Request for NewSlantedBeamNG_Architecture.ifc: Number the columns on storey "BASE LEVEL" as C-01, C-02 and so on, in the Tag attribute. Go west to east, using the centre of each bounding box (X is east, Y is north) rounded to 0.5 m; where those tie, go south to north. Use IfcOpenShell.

First a look at what the model holds.

```python
import ifcopenshell
import ifcopenshell.util.element
import ifcopenshell.util.placement

model = ifcopenshell.open("NewSlantedBeamNG_Architecture.ifc")
print(model.schema)
storey = next(s for s in model.by_type("IfcBuildingStorey") if s.Name == "BASE LEVEL")
columns = [e for e in ifcopenshell.util.element.get_decomposition(storey) if e.is_a("IfcColumn")]
for e in sorted(columns, key=lambda e: e.id()):
    origin = ifcopenshell.util.placement.get_local_placement(e.ObjectPlacement)[:3, 3]
    print(e.id(), e.Tag, e.Name, origin.round(2) + 0.0, sep=" | ")
```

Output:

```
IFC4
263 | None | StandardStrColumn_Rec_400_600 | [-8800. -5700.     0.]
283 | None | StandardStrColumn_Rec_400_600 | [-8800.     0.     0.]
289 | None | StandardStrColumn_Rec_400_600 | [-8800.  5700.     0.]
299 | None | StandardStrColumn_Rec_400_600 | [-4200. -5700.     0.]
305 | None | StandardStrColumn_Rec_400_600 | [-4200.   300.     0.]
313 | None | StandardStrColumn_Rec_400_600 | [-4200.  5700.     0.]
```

```python
import ifcopenshell
import ifcopenshell.geom
import ifcopenshell.util.element
import ifcopenshell.util.shape

model = ifcopenshell.open("NewSlantedBeamNG_Architecture.ifc")
settings = ifcopenshell.geom.settings()
settings.set("use-world-coords", True)


def centre(element):
    shape = ifcopenshell.geom.create_shape(settings, element)
    return ifcopenshell.util.shape.get_bbox_centroid(shape.geometry)


storey = next(s for s in model.by_type("IfcBuildingStorey") if s.Name == "BASE LEVEL")
columns = [e for e in ifcopenshell.util.element.get_decomposition(storey) if e.is_a("IfcColumn")]

# Insertion points can sit at a corner or the storey origin, so sort by the geometry (in metres).
centres = {e: centre(e) for e in columns}
columns.sort(key=lambda e: (round(centres[e][0] / 0.5), centres[e][1]))

for i, e in enumerate(columns, start=1):
    number = f"C-{i:02d}"
    e.Tag = number
    print(e.id(), number)

model.write("NewSlantedBeamNG_Architecture_rev.ifc")
```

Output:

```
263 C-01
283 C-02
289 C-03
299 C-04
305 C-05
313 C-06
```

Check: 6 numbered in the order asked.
